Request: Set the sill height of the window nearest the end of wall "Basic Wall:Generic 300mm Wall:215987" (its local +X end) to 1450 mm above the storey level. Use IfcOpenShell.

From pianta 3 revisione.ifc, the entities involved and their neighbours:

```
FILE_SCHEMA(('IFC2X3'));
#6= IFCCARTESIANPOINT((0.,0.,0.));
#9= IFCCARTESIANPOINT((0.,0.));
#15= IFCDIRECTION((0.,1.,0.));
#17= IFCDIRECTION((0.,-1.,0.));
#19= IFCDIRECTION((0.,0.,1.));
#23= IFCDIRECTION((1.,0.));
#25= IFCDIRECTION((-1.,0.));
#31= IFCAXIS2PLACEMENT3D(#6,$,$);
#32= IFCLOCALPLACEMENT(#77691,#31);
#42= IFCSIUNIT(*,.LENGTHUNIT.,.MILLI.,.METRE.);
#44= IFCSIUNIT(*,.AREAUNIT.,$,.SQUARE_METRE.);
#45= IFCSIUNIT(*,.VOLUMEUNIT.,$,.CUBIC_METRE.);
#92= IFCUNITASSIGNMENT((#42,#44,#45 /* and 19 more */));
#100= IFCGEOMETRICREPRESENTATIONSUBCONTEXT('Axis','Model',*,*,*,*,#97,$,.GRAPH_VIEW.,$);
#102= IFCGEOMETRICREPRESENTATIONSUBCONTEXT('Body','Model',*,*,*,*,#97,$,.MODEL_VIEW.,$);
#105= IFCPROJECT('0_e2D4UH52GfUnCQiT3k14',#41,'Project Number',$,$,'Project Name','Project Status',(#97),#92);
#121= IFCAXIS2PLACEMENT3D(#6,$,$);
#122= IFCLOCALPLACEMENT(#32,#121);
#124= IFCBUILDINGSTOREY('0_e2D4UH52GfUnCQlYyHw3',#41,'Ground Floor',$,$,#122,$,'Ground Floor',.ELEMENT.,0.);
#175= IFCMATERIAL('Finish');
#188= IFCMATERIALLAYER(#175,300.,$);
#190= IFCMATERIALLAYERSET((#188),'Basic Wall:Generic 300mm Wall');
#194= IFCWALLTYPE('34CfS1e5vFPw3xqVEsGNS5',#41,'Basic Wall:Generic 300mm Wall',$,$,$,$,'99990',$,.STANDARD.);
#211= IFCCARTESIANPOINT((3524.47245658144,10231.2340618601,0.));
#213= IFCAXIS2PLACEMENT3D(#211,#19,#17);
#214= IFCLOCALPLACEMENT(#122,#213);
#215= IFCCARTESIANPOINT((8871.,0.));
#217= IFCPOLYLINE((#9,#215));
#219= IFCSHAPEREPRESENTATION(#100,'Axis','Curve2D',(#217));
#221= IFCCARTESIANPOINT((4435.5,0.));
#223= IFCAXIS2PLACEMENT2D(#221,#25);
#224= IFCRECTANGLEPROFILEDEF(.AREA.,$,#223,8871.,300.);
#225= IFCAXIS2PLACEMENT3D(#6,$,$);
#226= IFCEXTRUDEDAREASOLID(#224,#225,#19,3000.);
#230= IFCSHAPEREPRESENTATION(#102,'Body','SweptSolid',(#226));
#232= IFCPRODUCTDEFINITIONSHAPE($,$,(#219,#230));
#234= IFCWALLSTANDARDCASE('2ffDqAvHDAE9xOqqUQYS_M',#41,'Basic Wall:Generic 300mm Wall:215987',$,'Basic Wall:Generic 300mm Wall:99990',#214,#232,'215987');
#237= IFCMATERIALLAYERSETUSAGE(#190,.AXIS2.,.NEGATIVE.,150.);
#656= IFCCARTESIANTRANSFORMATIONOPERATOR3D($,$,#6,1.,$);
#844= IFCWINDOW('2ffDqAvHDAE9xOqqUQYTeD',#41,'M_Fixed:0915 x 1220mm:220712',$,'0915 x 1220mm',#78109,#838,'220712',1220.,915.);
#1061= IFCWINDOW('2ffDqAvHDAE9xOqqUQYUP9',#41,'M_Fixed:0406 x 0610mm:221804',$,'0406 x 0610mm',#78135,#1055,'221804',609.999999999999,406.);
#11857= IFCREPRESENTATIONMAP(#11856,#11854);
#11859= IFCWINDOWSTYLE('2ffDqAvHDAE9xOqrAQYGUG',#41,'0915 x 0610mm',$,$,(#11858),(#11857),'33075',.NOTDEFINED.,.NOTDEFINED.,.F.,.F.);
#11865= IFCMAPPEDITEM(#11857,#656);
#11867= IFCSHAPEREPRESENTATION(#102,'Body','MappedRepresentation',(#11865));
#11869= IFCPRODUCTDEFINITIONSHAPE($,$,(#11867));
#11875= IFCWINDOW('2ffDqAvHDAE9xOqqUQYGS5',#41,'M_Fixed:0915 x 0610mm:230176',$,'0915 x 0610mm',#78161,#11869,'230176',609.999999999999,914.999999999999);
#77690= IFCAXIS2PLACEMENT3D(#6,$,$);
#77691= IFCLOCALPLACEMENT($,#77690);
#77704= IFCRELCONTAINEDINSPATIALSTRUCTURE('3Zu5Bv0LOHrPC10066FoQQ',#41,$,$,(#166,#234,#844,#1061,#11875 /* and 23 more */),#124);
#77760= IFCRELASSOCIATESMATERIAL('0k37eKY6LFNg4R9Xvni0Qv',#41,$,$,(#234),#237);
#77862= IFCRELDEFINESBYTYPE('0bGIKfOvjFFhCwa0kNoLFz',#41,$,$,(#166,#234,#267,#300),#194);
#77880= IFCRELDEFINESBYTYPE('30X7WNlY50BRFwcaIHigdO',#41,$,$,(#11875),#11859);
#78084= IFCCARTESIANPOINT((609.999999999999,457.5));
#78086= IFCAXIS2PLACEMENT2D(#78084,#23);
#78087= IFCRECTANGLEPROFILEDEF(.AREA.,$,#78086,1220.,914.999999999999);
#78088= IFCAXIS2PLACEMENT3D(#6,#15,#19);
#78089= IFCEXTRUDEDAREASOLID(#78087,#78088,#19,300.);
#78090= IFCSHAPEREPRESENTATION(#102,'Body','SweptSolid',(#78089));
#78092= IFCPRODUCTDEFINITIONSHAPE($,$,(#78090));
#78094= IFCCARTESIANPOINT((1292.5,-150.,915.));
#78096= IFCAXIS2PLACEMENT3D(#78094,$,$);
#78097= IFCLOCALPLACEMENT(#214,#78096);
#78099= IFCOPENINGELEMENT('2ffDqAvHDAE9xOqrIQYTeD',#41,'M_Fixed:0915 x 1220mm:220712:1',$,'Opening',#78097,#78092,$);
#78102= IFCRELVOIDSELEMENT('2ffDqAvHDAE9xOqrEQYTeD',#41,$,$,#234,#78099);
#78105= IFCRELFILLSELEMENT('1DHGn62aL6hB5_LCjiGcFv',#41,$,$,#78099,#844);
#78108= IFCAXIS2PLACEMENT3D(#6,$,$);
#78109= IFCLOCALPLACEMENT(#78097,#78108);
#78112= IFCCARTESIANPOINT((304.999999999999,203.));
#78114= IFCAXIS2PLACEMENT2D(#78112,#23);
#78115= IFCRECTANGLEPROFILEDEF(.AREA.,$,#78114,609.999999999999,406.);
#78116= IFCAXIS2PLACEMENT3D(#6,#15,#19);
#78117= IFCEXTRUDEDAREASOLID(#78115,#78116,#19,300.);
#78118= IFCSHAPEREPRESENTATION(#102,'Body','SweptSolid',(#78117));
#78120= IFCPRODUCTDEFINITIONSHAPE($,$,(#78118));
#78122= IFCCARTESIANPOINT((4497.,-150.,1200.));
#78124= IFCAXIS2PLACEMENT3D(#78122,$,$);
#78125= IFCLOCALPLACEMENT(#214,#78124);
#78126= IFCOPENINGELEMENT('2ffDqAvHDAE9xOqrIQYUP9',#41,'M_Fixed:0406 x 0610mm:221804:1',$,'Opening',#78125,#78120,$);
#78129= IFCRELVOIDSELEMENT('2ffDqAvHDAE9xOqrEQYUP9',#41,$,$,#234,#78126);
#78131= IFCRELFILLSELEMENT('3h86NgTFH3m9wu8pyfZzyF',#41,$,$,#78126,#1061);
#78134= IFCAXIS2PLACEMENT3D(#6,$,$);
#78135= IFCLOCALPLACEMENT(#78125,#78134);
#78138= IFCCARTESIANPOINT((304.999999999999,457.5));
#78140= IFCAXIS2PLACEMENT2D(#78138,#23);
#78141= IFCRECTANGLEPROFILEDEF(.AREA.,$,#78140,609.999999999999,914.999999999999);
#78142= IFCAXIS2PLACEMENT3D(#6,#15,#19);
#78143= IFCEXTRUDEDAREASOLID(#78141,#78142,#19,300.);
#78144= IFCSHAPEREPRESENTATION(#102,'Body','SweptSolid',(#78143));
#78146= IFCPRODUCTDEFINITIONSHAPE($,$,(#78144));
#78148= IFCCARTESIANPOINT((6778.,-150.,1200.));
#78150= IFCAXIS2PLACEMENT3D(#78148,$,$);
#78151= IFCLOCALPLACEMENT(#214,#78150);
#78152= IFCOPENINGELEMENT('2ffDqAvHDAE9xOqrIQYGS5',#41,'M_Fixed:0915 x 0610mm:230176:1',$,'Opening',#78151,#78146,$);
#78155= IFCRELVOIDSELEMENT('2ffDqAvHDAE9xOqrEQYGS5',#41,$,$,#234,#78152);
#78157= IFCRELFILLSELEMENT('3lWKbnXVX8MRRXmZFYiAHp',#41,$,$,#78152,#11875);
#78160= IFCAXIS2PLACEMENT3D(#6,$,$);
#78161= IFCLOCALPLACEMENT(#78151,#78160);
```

```python
import numpy as np
import ifcopenshell
import ifcopenshell.api.geometry
import ifcopenshell.geom
import ifcopenshell.util.element
import ifcopenshell.util.placement
import ifcopenshell.util.shape
import ifcopenshell.util.unit

model = ifcopenshell.open("pianta 3 revisione.ifc")
unit_scale = ifcopenshell.util.unit.calculate_unit_scale(model)

window = model.by_guid("2ffDqAvHDAE9xOqqUQYGS5")
opening = window.FillsVoids[0].RelatingOpeningElement
storey = ifcopenshell.util.element.get_container(window, ifc_class="IfcBuildingStorey")
level = ifcopenshell.util.placement.get_local_placement(storey.ObjectPlacement)[2, 3]

# The opening's origin need not be at the sill, so measure its lowest point.
shape = ifcopenshell.geom.create_shape(ifcopenshell.geom.settings(), opening)
bottom = ifcopenshell.util.shape.get_shape_bottom_elevation(shape, shape.geometry) / unit_scale
dz = level + 1.45 / unit_scale - bottom

shift = np.array([0.0, 0.0, dz])
# The window is placed relative to its opening, so it follows when the opening moves.
matrix = ifcopenshell.util.placement.get_local_placement(opening.ObjectPlacement)
matrix[:3, 3] += shift
ifcopenshell.api.geometry.edit_object_placement(
    model, product=opening, matrix=matrix, is_si=False, should_transform_children=True
)

print(f"moved by {dz * unit_scale:+.3f} m")

model.write("pianta 3 revisione-out.ifc")
```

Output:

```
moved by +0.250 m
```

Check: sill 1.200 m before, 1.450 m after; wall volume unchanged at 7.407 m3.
